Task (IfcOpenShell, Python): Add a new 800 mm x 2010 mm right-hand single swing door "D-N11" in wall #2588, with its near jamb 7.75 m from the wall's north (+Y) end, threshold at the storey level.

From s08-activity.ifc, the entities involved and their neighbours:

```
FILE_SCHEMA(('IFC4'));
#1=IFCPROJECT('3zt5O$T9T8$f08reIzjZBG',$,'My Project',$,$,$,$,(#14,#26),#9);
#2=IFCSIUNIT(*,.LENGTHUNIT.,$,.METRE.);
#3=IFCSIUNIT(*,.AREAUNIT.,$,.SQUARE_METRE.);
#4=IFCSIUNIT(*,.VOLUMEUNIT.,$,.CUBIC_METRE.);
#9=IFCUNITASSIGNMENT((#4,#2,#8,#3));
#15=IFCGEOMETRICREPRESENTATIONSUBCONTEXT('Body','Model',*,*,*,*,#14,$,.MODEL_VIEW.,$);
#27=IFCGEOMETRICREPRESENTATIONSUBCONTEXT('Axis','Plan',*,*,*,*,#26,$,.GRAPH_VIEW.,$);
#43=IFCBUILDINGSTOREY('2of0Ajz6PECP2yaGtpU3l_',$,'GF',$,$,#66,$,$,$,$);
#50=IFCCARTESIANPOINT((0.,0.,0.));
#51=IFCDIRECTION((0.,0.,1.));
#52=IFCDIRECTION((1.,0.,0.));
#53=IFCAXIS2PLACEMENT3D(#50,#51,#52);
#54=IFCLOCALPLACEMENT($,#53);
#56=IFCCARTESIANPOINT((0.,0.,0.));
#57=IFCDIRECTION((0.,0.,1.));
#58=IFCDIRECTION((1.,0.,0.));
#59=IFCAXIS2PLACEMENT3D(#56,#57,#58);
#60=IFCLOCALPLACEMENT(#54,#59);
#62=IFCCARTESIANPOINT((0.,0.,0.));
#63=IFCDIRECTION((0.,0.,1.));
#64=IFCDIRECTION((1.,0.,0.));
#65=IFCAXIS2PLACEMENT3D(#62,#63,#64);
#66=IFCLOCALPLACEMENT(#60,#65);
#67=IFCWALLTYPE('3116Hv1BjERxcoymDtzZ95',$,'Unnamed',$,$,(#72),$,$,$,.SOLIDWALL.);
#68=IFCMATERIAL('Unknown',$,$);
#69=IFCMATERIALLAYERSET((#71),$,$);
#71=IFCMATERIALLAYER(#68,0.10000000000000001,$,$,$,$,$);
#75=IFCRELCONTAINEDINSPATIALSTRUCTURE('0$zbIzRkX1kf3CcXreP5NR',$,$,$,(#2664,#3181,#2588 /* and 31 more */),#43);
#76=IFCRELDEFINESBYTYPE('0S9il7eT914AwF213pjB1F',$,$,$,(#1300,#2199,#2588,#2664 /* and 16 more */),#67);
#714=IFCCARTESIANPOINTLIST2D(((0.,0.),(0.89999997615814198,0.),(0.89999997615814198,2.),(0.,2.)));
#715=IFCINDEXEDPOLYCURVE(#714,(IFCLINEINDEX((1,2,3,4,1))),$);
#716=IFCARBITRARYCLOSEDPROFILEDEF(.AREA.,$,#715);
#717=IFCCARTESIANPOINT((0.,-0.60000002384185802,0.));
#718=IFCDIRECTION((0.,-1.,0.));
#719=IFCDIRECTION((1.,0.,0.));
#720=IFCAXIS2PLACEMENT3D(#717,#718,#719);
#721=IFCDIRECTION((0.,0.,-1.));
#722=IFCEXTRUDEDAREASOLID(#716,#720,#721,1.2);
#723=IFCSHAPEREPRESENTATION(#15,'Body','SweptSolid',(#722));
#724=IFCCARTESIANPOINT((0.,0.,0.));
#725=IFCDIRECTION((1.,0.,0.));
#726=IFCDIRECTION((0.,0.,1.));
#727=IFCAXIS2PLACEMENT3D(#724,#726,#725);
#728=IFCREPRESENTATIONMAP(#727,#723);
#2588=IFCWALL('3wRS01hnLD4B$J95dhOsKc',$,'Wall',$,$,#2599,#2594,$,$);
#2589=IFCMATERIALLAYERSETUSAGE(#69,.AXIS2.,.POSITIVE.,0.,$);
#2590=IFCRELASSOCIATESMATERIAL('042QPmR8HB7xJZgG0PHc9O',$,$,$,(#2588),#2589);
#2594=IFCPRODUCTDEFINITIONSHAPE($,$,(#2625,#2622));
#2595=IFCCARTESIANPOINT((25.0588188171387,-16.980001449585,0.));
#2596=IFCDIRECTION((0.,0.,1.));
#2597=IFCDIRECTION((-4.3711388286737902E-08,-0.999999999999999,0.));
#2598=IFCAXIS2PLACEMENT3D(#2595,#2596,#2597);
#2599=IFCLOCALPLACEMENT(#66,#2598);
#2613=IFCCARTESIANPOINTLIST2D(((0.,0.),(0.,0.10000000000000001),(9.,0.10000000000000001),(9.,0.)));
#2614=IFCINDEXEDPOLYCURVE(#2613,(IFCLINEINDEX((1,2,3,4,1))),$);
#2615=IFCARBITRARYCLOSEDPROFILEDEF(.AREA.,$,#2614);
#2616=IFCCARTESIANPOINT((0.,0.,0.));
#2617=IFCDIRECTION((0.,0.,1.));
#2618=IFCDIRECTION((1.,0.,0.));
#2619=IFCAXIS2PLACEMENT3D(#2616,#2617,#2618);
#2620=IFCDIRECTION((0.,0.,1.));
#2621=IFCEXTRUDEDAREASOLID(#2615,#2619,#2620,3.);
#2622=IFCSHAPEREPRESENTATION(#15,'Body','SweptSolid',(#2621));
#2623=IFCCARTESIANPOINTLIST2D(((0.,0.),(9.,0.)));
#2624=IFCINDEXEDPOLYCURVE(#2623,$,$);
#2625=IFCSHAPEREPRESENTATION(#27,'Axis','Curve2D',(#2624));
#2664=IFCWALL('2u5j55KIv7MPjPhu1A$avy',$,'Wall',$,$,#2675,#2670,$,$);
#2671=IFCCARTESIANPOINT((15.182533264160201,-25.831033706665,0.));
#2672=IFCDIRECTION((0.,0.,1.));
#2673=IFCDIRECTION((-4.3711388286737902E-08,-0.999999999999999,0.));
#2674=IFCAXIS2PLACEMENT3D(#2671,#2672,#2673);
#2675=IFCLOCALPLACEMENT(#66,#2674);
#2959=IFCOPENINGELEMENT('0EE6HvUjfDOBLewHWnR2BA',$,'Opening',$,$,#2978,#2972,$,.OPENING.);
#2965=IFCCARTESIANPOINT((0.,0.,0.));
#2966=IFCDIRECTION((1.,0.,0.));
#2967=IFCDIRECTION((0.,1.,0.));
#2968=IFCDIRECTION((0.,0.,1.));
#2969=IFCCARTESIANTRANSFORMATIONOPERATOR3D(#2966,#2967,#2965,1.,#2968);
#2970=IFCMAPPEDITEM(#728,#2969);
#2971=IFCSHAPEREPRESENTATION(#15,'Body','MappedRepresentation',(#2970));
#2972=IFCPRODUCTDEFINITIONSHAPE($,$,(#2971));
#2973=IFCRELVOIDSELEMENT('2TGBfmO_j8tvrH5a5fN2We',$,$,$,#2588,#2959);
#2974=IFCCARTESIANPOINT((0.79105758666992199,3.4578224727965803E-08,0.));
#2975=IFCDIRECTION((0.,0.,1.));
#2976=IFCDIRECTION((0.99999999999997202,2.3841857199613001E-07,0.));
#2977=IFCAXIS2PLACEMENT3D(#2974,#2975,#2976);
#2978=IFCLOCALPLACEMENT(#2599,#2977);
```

```python
import numpy as np
import ifcopenshell
import ifcopenshell.api.feature
import ifcopenshell.api.geometry
import ifcopenshell.api.root
import ifcopenshell.api.spatial
import ifcopenshell.geom
import ifcopenshell.util.element
import ifcopenshell.util.placement
import ifcopenshell.util.representation
import ifcopenshell.util.shape
import ifcopenshell.util.unit

model = ifcopenshell.open("s08-activity.ifc")
unit_scale = ifcopenshell.util.unit.calculate_unit_scale(model)
settings = ifcopenshell.geom.settings()


def volume(element):
    """Net volume in cubic metres, openings subtracted."""
    shape = ifcopenshell.geom.create_shape(settings, element)
    return ifcopenshell.util.shape.get_volume(shape.geometry)


wall = model.by_id(2588)
storey = ifcopenshell.util.element.get_container(wall, ifc_class="IfcBuildingStorey")
context = ifcopenshell.util.representation.get_context(model, "Model", "Body", "MODEL_VIEW")
before = volume(wall)

width, height, from_end, sill = 0.8, 2.01, 7.75, 0.0  # metres

# The wall runs along its own X axis, and the end named is its -X end.
wall_shape = ifcopenshell.geom.create_shape(settings, wall)
x, y, z = ifcopenshell.util.shape.get_vertices(wall_shape.geometry).T
start = x.min() + from_end
face, thickness = float(y.min()), float(y.max() - y.min())
wall_matrix = ifcopenshell.util.placement.get_local_placement(wall.ObjectPlacement)
level = ifcopenshell.util.placement.get_local_placement(storey.ObjectPlacement)[2, 3]


def in_wall(x, y):
    """Placement at x, y metres in the wall's axes, at sill height."""
    matrix = wall_matrix.copy()
    matrix[:, 3] = wall_matrix @ np.array([x / unit_scale, y / unit_scale, 0.0, 1.0])
    matrix[2, 3] = level + sill / unit_scale
    return matrix


# Opening: a box that overshoots both wall faces by 50 mm.
opening = ifcopenshell.api.root.create_entity(model, ifc_class="IfcOpeningElement", predefined_type="OPENING")
box = ifcopenshell.api.geometry.add_wall_representation(
    model, context=context, length=width, height=height, thickness=thickness + 0.1
)
ifcopenshell.api.geometry.assign_representation(model, product=opening, representation=box)
ifcopenshell.api.geometry.edit_object_placement(model, product=opening, matrix=in_wall(start, face - 0.05), is_si=False)
ifcopenshell.api.feature.add_feature(model, feature=opening, element=wall)

door = ifcopenshell.api.root.create_entity(model, ifc_class="IfcDoor", name="D-N11", predefined_type="DOOR")
door.OverallWidth, door.OverallHeight = width / unit_scale, height / unit_scale
door.OperationType = "SINGLE_SWING_RIGHT"
body = ifcopenshell.api.geometry.add_door_representation(
    model,
    context=context,
    overall_width=door.OverallWidth,
    overall_height=door.OverallHeight,
    operation_type="SINGLE_SWING_RIGHT",
    lining_properties={"LiningDepth": thickness / unit_scale, "ThresholdDepth": thickness / unit_scale},
)
ifcopenshell.api.geometry.assign_representation(model, product=door, representation=body)
ifcopenshell.api.spatial.assign_container(model, products=[door], relating_structure=storey)
ifcopenshell.api.feature.add_filling(model, opening=opening, element=door)

# The lining spans the wall, so the door starts at the wall face.
ifcopenshell.api.geometry.edit_object_placement(model, product=door, matrix=in_wall(start, face), is_si=False)

after = volume(wall)

print(f"wall volume {before:.3f} -> {after:.3f} m3")

model.write("s08-activity-out.ifc")
```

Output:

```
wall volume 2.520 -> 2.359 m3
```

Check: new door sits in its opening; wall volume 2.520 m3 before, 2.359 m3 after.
